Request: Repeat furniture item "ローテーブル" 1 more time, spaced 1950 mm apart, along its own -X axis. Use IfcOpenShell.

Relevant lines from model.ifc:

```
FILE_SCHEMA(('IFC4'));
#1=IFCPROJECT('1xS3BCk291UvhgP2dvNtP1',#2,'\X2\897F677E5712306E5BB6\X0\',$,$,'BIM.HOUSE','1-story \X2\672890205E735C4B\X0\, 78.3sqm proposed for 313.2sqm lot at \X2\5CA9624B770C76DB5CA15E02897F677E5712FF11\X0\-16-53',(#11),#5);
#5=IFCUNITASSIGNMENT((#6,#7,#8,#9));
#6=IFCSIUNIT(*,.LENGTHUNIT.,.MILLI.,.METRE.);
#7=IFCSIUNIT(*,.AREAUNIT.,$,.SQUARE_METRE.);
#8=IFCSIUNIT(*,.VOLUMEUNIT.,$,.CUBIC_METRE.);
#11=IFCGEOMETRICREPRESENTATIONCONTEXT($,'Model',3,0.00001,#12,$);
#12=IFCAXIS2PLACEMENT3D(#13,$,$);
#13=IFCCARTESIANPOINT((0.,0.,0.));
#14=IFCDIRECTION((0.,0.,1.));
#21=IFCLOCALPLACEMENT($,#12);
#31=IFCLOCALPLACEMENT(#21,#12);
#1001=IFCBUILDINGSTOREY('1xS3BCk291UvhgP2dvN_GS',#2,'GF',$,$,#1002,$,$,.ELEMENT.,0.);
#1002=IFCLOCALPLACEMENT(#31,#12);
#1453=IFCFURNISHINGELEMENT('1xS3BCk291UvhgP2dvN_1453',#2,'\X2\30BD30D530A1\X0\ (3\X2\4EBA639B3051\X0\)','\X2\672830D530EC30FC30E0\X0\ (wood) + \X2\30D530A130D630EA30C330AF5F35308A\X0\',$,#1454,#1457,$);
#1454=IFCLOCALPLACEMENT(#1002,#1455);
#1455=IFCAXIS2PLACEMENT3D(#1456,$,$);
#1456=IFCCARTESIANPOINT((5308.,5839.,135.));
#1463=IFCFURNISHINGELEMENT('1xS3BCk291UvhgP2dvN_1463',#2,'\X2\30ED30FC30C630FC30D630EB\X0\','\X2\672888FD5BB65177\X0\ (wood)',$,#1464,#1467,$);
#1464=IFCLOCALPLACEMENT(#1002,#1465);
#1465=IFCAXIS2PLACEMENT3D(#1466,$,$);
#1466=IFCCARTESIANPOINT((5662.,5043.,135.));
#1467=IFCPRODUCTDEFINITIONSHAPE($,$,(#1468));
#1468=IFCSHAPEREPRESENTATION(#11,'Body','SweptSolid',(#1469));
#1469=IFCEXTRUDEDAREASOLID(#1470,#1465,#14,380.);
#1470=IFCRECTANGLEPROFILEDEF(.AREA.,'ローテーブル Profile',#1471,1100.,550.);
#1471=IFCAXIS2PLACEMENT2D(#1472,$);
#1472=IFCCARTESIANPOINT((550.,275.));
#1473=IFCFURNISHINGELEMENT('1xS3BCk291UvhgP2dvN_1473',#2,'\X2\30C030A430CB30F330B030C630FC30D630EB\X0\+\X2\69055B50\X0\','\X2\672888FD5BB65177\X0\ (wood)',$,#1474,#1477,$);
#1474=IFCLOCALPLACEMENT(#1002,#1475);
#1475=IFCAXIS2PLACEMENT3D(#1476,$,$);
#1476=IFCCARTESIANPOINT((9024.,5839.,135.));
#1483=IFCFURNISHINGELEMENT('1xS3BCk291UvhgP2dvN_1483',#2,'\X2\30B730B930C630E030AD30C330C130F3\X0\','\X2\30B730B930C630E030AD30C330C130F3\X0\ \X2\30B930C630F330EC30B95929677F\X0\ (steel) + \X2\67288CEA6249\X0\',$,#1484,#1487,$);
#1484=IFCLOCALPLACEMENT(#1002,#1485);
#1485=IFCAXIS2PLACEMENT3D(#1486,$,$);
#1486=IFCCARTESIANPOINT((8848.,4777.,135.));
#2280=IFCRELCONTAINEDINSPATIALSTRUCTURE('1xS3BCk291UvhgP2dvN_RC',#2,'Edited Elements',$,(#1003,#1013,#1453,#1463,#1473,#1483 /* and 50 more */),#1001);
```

```python
import ifcopenshell
import ifcopenshell.api.geometry
import ifcopenshell.api.root
import ifcopenshell.util.element
import ifcopenshell.util.placement

model = ifcopenshell.open("model.ifc")


def reuse_history(source, copy):
    """copy_class also copies each property set's owner history, people and application; keep the originals."""
    for rel in copy.IsDefinedBy:
        if rel.is_a("IfcRelDefinesByProperties") and (history := rel.RelatingPropertyDefinition.OwnerHistory):
            rel.RelatingPropertyDefinition.OwnerHistory = source.OwnerHistory
            ifcopenshell.util.element.remove_deep2(model, history)


source = model.by_guid("1xS3BCk291UvhgP2dvN_1463")
base = ifcopenshell.util.placement.get_local_placement(source.ObjectPlacement)
step = -base[:3, 0] * 1950.0

for i in range(1, 2):
    copy = ifcopenshell.api.root.copy_class(model, product=source)
    copy.Representation = ifcopenshell.util.element.copy_deep(
        model, source.Representation, exclude=["IfcGeometricRepresentationContext", "IfcRepresentationMap"]
    )
    reuse_history(source, copy)
    matrix = base.copy()
    matrix[:3, 3] += i * step
    print("added at", matrix[:3, 3].round(3) + 0.0)
    ifcopenshell.api.geometry.edit_object_placement(model, product=copy, matrix=matrix, is_si=False)

model.write("model_edited.ifc")
```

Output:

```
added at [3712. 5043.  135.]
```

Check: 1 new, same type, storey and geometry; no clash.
